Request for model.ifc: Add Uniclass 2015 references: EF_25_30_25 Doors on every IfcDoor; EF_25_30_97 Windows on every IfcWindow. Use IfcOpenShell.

First a look at what the model holds.

```python
import ifcopenshell

model = ifcopenshell.open("model.ifc")
print(model.schema)
print("classifications:", [c.Name for c in model.by_type("IfcClassification")])
for ifc_class in ("IfcDoor", "IfcRoof", "IfcStair", "IfcWall", "IfcWindow"):
    print(ifc_class, len(model.by_type(ifc_class)))
```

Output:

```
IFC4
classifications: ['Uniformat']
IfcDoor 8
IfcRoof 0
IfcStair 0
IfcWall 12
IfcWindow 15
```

```python
import ifcopenshell
import ifcopenshell.api.classification

model = ifcopenshell.open("model.ifc")

system = ifcopenshell.api.classification.add_classification(model, classification="Uniclass 2015")

codes = {
    "IfcDoor": ("EF_25_30_25", "Doors"),
    "IfcWindow": ("EF_25_30_97", "Windows"),
}
for ifc_class, (code, name) in codes.items():
    products = model.by_type(ifc_class)
    ifcopenshell.api.classification.add_reference(
        model, products=products, classification=system, identification=code, name=name
    )
    print(code, len(products))

model.write("model_v2.ifc")
```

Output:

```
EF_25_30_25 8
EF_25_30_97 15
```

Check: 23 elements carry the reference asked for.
